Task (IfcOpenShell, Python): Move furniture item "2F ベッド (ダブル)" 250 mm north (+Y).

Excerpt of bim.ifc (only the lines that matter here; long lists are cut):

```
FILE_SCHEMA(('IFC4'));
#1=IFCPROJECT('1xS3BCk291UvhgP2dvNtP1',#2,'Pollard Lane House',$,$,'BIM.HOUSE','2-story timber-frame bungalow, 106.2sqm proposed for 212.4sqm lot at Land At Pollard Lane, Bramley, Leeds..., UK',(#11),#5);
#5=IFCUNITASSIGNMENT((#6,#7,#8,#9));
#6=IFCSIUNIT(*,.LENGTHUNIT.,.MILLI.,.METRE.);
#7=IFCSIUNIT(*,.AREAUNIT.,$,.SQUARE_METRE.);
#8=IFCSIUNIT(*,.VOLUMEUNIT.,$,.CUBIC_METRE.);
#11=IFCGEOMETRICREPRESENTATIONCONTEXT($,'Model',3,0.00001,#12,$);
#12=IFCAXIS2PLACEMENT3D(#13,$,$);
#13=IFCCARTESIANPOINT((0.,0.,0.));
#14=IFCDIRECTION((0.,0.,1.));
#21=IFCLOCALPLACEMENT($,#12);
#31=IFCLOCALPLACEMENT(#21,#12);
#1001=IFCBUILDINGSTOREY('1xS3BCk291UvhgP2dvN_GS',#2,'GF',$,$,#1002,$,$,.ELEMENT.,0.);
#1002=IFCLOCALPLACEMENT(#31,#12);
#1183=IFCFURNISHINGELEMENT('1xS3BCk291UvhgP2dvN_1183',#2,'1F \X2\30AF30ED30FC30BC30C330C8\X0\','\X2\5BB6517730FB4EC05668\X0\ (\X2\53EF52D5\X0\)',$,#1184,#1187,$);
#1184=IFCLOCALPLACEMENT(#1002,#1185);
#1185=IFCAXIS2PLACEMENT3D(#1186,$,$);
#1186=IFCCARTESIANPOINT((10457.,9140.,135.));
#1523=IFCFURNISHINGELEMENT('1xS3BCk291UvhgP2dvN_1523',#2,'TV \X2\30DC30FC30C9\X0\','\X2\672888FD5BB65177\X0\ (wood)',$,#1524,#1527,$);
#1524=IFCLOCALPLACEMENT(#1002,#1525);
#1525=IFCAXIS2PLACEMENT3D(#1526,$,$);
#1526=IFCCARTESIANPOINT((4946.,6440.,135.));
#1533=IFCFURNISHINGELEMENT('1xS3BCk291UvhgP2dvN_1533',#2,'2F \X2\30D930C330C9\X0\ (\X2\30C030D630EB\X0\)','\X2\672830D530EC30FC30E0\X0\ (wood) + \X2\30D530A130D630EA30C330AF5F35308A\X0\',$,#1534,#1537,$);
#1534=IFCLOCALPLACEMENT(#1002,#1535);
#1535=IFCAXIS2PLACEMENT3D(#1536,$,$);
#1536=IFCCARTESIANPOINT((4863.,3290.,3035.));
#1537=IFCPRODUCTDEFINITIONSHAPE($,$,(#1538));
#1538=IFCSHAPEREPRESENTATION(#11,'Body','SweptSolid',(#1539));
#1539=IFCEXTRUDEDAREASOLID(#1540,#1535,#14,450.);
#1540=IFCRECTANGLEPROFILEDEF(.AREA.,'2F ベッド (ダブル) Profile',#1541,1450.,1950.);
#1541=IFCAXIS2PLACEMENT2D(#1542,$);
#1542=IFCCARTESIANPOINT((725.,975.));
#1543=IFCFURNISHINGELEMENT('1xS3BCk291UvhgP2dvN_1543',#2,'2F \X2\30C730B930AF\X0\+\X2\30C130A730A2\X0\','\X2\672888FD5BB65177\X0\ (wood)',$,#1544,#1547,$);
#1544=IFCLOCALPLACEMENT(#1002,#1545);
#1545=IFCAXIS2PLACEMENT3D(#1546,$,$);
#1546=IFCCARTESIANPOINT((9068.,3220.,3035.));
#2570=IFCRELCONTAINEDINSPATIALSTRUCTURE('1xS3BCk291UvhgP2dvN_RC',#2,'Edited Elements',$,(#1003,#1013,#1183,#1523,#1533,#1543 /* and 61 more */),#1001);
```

```python
import ifcopenshell
import ifcopenshell.api.geometry
import ifcopenshell.util.placement
import ifcopenshell.util.unit

model = ifcopenshell.open("bim.ifc")
unit_scale = ifcopenshell.util.unit.calculate_unit_scale(model)

item = model.by_id(1533)
matrix = ifcopenshell.util.placement.get_local_placement(item.ObjectPlacement)
matrix[1, 3] += 0.25 / unit_scale
ifcopenshell.api.geometry.edit_object_placement(model, product=item, matrix=matrix, is_si=False)

print(ifcopenshell.util.placement.get_local_placement(item.ObjectPlacement).round(3) + 0.0)

model.write("bim-out.ifc")
```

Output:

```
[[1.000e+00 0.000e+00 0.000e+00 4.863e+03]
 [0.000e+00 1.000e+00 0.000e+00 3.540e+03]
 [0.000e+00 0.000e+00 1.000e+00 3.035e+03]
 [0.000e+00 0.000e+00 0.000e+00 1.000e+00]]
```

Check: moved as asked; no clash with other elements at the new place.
